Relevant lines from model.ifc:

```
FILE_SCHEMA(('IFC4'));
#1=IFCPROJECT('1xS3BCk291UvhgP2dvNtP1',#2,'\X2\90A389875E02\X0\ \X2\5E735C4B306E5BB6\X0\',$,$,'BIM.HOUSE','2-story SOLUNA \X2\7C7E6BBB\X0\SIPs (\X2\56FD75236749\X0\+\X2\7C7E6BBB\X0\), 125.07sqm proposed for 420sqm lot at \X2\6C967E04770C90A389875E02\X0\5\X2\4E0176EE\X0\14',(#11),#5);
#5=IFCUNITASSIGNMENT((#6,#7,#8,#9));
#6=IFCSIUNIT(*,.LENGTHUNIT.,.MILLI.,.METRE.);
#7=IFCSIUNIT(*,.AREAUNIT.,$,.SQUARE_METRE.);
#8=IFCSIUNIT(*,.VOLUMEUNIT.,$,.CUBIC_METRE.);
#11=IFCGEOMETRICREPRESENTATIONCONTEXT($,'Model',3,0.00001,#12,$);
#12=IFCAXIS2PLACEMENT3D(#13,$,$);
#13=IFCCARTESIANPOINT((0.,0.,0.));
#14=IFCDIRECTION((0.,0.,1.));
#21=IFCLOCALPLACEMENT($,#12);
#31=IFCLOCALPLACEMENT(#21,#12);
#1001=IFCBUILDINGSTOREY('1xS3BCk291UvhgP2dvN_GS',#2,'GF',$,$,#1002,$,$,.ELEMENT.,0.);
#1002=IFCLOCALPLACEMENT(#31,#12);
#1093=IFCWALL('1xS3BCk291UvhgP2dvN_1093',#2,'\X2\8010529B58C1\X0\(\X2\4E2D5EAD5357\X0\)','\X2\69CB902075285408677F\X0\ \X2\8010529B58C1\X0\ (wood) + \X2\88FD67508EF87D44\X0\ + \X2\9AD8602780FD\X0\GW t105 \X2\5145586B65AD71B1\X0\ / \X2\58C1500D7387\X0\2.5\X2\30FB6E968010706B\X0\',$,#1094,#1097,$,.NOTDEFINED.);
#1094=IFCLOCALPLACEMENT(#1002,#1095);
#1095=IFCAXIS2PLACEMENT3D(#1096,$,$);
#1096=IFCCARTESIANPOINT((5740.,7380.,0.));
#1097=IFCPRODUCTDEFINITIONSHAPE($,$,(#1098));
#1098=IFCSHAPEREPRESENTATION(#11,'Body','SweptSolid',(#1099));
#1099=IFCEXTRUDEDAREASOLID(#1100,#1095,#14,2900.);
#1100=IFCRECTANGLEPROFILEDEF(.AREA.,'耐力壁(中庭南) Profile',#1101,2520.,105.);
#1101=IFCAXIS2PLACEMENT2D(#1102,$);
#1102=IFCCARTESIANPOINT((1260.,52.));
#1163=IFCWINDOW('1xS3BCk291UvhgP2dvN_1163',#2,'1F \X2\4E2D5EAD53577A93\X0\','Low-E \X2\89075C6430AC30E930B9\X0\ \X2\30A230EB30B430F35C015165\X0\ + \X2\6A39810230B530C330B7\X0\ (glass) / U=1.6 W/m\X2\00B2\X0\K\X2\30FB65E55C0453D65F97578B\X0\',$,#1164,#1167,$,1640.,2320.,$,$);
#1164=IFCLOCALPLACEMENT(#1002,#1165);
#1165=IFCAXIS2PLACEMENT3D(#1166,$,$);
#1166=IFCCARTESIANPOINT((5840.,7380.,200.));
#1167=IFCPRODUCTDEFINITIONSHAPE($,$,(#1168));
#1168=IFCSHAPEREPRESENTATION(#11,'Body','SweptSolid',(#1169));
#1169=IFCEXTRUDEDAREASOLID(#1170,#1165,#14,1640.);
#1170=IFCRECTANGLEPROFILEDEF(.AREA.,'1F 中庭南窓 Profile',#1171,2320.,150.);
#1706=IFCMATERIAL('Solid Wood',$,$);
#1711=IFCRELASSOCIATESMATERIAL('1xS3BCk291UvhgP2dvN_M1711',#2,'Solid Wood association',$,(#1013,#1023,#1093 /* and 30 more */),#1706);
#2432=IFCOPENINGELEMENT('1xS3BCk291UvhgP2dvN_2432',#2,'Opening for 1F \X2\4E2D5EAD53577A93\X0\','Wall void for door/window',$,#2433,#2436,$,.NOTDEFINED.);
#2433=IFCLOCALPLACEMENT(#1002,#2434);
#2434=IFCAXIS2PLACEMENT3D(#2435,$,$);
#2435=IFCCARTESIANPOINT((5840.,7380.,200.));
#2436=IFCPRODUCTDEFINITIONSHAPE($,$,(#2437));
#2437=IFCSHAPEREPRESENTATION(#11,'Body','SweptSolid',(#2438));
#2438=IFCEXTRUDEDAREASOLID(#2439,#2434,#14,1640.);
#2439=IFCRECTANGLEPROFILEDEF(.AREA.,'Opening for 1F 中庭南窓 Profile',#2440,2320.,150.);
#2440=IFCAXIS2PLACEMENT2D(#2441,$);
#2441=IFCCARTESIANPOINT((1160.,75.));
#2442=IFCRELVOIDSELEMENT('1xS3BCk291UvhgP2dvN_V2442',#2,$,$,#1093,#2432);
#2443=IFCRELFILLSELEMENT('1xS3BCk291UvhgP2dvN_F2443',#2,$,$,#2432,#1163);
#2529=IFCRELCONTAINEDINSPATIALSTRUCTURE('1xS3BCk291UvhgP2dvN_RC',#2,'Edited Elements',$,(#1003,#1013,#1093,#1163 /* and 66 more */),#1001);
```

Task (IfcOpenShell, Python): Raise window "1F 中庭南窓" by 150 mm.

```python
import numpy as np
import ifcopenshell
import ifcopenshell.api.geometry
import ifcopenshell.util.placement
import ifcopenshell.util.unit

model = ifcopenshell.open("model.ifc")
unit_scale = ifcopenshell.util.unit.calculate_unit_scale(model)

window = model.by_guid("1xS3BCk291UvhgP2dvN_1163")
opening = window.FillsVoids[0].RelatingOpeningElement
dz = 0.15 / unit_scale

shift = np.array([0.0, 0.0, dz])
# The window is not placed relative to its opening, so move both.
for product in (opening, window):
    matrix = ifcopenshell.util.placement.get_local_placement(product.ObjectPlacement)
    matrix[:3, 3] += shift
    ifcopenshell.api.geometry.edit_object_placement(model, product=product, matrix=matrix, is_si=False)

print(f"moved by {dz * unit_scale:+.3f} m")

model.write("model_edited.ifc")
```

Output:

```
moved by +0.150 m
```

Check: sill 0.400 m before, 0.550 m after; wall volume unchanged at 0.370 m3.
